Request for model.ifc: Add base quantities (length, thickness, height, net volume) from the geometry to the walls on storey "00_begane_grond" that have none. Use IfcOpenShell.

First a look at what the model holds.

```python
import ifcopenshell
import ifcopenshell.util.element
import ifcopenshell.util.unit

model = ifcopenshell.open("model.ifc")
print(model.schema)
for unit_type in ("LENGTHUNIT", "AREAUNIT", "VOLUMEUNIT"):
    print(unit_type, ifcopenshell.util.unit.calculate_unit_scale(model, unit_type))
storey = next(s for s in model.by_type("IfcBuildingStorey") if s.Name == "00_begane_grond")
walls = [e for e in ifcopenshell.util.element.get_decomposition(storey) if e.is_a("IfcWall")]
for e in sorted(walls, key=lambda e: e.id()):
    print(e.id(), e.is_a(), e.Name, list(ifcopenshell.util.element.get_psets(e, qtos_only=True)), sep=" | ")
```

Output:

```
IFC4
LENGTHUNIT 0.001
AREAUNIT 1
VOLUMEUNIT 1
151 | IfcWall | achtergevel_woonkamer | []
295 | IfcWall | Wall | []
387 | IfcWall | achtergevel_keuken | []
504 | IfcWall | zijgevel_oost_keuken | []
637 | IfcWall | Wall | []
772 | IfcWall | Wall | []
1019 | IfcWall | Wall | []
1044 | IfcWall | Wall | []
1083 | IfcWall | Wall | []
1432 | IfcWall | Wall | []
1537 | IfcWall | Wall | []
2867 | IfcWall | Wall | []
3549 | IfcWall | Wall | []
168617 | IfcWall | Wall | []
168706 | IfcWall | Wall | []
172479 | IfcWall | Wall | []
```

```python
import ifcopenshell
import ifcopenshell.api.pset
import ifcopenshell.geom
import ifcopenshell.util.element
import ifcopenshell.util.shape
import ifcopenshell.util.unit

model = ifcopenshell.open("model.ifc")
unit_scale = ifcopenshell.util.unit.calculate_unit_scale(model)
volume_scale = ifcopenshell.util.unit.calculate_unit_scale(model, "VOLUMEUNIT")
settings = ifcopenshell.geom.settings()

storey = next(s for s in model.by_type("IfcBuildingStorey") if s.Name == "00_begane_grond")
walls = [e for e in ifcopenshell.util.element.get_decomposition(storey) if e.is_a("IfcWall")]

for e in sorted(walls, key=lambda e: e.id()):
    if ifcopenshell.util.element.get_psets(e, qtos_only=True, should_inherit=False):
        continue
    # Geometry comes back in metres, in the element's own axes.
    shape = ifcopenshell.geom.create_shape(settings, e)
    values = {
        "Length": ifcopenshell.util.shape.get_x(shape.geometry) / unit_scale,
        "Width": ifcopenshell.util.shape.get_y(shape.geometry) / unit_scale,
        "Height": ifcopenshell.util.shape.get_z(shape.geometry) / unit_scale,
        "NetVolume": ifcopenshell.util.shape.get_volume(shape.geometry) / volume_scale,
    }
    qto = ifcopenshell.api.pset.add_qto(model, product=e, name="Qto_WallBaseQuantities")
    ifcopenshell.api.pset.edit_qto(model, qto=qto, properties=values)
    print(e.id(), {k: round(v, 3) for k, v in values.items()})

model.write("model-out.ifc")
```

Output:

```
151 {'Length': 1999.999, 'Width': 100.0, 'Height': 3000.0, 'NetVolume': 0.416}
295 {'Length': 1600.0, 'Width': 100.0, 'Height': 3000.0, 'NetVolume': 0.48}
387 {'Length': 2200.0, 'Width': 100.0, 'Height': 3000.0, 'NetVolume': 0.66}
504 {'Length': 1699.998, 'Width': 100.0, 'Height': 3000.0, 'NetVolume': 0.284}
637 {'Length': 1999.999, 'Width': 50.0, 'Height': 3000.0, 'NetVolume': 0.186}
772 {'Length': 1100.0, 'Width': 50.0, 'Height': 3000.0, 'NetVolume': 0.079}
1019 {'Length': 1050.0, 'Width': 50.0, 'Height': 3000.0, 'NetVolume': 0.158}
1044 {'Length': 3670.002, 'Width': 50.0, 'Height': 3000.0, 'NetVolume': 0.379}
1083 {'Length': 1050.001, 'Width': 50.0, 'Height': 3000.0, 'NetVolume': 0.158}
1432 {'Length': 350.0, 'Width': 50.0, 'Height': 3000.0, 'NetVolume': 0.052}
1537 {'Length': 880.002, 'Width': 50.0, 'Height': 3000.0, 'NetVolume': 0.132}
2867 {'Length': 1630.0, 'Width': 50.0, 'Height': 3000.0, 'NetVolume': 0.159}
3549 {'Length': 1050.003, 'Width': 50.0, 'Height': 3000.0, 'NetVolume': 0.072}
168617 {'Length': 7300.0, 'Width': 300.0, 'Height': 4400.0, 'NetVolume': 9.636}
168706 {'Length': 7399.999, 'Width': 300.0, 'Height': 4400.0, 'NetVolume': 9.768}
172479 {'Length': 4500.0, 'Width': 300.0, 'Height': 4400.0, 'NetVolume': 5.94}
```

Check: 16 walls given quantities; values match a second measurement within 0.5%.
